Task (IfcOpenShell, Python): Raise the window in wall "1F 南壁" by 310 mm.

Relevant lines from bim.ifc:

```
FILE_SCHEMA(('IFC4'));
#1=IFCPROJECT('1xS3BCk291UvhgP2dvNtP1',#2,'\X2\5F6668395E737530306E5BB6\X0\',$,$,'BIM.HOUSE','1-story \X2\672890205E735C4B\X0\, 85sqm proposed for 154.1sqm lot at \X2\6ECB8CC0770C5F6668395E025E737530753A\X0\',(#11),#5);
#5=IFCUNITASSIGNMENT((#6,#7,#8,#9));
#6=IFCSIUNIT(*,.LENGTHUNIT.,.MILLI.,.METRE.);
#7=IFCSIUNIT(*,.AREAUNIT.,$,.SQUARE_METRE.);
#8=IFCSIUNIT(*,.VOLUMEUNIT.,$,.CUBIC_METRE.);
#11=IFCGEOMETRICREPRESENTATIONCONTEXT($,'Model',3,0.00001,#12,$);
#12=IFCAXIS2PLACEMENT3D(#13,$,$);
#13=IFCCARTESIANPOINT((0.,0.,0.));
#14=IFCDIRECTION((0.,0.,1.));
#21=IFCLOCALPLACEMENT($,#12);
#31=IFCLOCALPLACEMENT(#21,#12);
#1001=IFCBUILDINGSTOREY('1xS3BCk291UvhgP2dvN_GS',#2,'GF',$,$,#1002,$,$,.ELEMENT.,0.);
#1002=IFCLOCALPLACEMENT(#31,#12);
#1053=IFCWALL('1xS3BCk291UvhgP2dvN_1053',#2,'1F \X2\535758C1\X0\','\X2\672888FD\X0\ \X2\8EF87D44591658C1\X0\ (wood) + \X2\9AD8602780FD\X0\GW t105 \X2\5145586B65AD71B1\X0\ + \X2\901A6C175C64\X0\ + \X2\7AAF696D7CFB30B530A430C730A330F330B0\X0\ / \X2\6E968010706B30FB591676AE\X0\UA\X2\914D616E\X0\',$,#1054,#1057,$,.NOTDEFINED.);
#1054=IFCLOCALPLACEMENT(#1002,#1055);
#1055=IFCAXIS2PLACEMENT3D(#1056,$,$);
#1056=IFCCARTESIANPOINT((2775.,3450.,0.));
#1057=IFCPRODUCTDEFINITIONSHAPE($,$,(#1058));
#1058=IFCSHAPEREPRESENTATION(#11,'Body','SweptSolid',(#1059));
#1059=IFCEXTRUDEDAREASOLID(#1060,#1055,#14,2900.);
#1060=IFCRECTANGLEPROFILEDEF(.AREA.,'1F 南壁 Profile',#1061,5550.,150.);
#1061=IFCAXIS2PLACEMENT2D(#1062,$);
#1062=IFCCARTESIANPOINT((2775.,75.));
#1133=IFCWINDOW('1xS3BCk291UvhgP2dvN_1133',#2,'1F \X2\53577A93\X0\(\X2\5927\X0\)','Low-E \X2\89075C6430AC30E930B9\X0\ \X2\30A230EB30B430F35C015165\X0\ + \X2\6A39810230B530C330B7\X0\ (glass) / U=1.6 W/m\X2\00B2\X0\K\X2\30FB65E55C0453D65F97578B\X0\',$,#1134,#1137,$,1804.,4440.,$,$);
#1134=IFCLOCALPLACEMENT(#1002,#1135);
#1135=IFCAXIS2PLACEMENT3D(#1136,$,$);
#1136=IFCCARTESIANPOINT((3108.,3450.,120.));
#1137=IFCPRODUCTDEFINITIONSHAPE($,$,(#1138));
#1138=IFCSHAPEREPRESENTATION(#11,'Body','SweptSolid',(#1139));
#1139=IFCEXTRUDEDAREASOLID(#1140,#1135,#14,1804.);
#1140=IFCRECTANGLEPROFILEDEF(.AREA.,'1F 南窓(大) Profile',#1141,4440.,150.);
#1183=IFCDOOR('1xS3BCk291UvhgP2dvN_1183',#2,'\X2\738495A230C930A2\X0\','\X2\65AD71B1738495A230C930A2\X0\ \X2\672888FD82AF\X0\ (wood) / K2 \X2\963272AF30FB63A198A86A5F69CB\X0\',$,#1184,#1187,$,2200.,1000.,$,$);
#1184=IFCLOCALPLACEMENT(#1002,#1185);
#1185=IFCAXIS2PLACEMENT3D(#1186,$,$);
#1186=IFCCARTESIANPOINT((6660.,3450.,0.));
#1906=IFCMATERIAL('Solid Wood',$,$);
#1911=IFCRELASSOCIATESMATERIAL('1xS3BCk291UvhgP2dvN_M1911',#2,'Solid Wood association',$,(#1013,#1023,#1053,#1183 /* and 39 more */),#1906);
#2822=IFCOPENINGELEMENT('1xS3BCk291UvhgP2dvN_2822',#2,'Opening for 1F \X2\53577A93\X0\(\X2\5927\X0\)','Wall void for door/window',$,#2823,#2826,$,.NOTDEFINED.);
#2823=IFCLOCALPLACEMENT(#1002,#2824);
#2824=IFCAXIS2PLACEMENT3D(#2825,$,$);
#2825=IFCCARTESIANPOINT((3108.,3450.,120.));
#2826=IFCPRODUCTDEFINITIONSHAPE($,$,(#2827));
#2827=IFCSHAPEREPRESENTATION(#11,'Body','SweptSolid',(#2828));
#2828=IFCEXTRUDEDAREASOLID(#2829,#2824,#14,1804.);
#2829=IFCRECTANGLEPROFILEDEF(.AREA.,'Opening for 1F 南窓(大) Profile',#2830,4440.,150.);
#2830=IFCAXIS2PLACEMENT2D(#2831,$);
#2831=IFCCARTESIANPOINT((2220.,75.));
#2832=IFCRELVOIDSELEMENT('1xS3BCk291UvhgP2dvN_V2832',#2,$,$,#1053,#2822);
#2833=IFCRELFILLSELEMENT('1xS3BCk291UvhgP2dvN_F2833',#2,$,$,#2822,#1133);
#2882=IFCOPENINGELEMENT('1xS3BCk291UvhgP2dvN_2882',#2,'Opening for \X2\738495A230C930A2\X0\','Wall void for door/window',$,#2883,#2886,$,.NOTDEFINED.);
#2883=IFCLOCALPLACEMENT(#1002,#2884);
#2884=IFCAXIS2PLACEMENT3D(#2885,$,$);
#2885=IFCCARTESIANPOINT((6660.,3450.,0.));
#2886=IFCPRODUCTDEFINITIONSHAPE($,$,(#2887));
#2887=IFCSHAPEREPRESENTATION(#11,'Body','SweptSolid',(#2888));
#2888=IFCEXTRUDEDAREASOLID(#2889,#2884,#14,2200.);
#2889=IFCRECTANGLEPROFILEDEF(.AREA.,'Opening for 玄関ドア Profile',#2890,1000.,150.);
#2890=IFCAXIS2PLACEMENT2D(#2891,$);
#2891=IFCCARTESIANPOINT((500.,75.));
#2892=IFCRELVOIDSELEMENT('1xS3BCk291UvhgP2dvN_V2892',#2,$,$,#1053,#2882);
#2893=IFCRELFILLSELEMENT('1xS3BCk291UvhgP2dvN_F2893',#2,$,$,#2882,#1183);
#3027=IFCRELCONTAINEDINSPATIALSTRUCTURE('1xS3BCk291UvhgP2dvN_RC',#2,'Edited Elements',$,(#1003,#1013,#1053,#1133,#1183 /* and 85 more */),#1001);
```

```python
import numpy as np
import ifcopenshell
import ifcopenshell.api.geometry
import ifcopenshell.util.placement
import ifcopenshell.util.unit

model = ifcopenshell.open("bim.ifc")
unit_scale = ifcopenshell.util.unit.calculate_unit_scale(model)

window = model.by_guid("1xS3BCk291UvhgP2dvN_1133")
opening = window.FillsVoids[0].RelatingOpeningElement
dz = 310.0

shift = np.array([0.0, 0.0, dz])
# The window is not placed relative to its opening, so move both.
for product in (opening, window):
    matrix = ifcopenshell.util.placement.get_local_placement(product.ObjectPlacement)
    matrix[:3, 3] += shift
    ifcopenshell.api.geometry.edit_object_placement(model, product=product, matrix=matrix, is_si=False)

print(f"moved by {dz * unit_scale:+.3f} m")

model.write("bim_edited.ifc")
```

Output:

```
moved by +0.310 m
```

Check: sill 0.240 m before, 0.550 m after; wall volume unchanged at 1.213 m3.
